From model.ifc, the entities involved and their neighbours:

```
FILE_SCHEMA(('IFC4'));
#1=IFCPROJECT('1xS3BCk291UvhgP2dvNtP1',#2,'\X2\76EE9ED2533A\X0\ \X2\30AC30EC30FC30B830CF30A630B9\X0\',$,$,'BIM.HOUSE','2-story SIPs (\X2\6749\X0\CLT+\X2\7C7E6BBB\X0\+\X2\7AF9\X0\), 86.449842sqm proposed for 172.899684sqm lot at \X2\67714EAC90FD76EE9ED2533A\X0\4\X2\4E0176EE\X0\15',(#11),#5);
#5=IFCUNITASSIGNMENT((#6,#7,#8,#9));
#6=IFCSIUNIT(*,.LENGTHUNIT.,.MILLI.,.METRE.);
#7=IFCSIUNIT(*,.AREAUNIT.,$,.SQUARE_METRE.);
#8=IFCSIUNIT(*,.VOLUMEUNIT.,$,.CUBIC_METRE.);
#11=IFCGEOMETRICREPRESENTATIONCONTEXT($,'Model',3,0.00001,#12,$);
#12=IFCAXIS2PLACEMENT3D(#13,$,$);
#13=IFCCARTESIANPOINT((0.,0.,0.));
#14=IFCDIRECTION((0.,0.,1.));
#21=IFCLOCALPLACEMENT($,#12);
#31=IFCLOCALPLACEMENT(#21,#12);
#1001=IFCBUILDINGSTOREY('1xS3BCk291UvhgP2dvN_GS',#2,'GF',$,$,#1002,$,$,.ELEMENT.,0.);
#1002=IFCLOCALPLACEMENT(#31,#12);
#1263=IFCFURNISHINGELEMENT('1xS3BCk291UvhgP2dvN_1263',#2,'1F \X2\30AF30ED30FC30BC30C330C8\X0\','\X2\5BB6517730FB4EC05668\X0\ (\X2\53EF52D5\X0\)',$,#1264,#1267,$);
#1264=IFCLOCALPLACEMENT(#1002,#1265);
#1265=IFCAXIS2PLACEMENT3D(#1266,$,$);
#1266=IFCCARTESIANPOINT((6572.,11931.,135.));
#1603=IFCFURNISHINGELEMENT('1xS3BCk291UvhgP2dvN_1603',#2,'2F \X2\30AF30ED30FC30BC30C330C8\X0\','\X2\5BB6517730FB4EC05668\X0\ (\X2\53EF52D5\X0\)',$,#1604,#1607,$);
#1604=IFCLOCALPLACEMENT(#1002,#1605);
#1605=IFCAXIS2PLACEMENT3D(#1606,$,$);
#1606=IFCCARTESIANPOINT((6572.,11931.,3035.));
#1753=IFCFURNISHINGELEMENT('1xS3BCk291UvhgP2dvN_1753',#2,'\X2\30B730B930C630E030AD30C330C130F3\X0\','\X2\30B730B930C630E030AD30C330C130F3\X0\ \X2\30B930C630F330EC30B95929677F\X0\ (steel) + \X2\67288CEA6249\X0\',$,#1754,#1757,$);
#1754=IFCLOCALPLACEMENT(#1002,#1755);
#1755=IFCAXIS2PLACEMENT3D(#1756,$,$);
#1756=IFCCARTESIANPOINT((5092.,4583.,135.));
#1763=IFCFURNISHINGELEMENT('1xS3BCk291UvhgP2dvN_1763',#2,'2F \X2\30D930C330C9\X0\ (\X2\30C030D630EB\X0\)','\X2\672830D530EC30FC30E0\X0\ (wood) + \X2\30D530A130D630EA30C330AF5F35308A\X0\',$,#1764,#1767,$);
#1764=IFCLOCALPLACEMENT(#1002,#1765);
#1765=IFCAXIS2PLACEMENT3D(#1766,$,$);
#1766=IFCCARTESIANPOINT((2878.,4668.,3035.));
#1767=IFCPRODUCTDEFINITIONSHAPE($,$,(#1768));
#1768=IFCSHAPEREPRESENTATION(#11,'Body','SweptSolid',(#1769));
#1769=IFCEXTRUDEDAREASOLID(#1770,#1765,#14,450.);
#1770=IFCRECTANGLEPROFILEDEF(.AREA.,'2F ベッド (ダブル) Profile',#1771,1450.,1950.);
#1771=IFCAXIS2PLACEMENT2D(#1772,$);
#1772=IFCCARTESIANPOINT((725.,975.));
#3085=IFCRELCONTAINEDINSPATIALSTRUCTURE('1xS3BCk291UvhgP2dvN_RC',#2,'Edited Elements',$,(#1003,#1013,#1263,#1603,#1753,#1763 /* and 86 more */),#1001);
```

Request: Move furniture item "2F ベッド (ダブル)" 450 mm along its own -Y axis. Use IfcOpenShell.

```python
import ifcopenshell
import ifcopenshell.api.geometry
import ifcopenshell.util.placement
import ifcopenshell.util.unit

model = ifcopenshell.open("model.ifc")
unit_scale = ifcopenshell.util.unit.calculate_unit_scale(model)

item = model.by_guid("1xS3BCk291UvhgP2dvN_1763")
matrix = ifcopenshell.util.placement.get_local_placement(item.ObjectPlacement)
matrix[:3, 3] -= matrix[:3, 1] * 0.45 / unit_scale
ifcopenshell.api.geometry.edit_object_placement(model, product=item, matrix=matrix, is_si=False)

print(ifcopenshell.util.placement.get_local_placement(item.ObjectPlacement).round(3) + 0.0)

model.write("model_rev.ifc")
```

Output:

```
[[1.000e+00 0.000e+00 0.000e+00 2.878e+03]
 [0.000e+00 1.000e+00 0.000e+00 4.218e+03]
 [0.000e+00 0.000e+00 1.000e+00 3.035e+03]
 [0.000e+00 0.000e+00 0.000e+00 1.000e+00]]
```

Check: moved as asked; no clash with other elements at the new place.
